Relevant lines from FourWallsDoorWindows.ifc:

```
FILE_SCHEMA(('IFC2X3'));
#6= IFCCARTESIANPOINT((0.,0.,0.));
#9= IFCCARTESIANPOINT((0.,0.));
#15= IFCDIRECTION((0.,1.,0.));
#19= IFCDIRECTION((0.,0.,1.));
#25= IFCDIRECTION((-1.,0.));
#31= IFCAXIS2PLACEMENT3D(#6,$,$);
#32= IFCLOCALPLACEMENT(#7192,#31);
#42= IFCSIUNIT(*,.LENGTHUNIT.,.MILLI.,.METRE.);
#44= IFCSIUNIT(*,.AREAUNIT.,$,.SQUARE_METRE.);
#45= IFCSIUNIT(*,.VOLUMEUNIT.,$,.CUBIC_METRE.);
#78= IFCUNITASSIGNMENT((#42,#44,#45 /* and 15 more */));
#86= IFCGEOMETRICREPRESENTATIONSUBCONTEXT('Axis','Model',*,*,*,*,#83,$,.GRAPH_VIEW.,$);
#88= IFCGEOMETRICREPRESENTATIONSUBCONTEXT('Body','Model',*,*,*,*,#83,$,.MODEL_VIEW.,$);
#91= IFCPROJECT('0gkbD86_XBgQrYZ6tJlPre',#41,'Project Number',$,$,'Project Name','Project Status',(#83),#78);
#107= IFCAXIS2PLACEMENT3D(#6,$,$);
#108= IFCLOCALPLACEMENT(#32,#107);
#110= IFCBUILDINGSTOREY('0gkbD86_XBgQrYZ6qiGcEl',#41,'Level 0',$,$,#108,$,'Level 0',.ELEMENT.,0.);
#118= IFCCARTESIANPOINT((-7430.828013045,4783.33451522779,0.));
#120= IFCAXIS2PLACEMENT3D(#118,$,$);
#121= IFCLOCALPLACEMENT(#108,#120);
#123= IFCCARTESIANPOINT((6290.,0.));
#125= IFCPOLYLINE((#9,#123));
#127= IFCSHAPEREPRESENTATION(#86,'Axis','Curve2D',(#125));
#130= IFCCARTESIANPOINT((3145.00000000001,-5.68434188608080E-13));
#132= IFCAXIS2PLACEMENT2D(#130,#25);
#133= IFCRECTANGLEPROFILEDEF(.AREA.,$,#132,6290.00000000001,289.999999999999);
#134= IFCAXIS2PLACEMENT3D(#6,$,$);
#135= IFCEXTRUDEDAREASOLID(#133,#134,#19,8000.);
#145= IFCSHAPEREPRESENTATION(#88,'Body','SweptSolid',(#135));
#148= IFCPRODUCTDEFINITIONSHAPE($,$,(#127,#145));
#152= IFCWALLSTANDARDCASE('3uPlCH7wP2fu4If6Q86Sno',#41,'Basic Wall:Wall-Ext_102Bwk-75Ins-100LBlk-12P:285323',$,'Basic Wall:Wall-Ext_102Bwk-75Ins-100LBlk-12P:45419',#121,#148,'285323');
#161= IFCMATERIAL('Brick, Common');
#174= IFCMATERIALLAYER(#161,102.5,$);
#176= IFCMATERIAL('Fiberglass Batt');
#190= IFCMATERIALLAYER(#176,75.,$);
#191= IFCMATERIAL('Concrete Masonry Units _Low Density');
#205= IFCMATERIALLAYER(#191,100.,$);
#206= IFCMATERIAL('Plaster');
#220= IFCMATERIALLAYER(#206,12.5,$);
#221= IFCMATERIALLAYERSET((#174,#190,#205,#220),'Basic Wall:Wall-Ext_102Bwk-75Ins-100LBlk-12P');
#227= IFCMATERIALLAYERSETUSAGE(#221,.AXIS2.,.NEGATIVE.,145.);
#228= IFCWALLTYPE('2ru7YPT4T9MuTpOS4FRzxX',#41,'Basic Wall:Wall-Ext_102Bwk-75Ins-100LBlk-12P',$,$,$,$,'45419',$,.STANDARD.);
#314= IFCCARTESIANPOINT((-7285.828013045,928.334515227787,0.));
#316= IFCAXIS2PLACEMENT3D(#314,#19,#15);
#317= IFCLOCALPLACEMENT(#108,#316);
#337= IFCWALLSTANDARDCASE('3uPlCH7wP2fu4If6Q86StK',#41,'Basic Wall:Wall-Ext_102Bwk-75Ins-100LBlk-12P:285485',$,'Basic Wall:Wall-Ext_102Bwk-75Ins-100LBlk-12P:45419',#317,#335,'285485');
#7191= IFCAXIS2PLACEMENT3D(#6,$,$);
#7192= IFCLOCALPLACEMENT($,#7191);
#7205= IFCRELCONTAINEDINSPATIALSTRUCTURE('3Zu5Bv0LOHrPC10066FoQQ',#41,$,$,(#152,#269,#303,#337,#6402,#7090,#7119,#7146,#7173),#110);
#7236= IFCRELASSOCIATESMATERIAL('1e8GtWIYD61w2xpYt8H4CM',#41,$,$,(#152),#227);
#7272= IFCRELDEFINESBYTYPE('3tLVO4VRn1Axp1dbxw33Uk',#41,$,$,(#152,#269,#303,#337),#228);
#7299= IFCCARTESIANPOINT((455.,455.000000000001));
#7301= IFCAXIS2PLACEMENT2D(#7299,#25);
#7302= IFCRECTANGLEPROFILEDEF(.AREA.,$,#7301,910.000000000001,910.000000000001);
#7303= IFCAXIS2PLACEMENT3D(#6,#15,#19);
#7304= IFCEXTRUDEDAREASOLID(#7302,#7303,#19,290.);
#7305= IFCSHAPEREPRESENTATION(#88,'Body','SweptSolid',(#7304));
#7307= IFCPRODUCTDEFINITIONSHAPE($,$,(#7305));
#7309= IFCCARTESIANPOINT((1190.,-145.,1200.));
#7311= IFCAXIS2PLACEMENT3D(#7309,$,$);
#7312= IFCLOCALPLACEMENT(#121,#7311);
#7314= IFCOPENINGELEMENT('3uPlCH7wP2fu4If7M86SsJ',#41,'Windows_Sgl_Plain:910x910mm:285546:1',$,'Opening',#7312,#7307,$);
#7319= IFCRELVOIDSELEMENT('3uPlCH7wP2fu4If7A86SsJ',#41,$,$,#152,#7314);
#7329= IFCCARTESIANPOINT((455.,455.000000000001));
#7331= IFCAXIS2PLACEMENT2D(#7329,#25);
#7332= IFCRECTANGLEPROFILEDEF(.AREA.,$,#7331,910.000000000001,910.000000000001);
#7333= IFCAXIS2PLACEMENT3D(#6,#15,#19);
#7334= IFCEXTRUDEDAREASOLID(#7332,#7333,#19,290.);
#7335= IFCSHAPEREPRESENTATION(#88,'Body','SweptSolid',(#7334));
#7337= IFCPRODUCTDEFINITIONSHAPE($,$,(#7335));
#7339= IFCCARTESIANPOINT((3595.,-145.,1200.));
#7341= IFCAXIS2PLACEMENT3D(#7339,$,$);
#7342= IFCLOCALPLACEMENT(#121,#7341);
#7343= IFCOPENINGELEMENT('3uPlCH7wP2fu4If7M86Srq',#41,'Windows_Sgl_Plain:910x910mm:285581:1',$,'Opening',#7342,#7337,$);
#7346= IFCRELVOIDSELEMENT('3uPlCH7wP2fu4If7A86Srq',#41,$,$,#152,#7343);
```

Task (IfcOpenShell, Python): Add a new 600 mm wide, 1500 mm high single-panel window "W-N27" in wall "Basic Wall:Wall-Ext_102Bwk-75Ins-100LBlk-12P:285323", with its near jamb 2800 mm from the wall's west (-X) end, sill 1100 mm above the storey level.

```python
import numpy as np
import ifcopenshell
import ifcopenshell.api.feature
import ifcopenshell.api.geometry
import ifcopenshell.api.root
import ifcopenshell.api.spatial
import ifcopenshell.api.type
import ifcopenshell.geom
import ifcopenshell.util.element
import ifcopenshell.util.placement
import ifcopenshell.util.representation
import ifcopenshell.util.shape
import ifcopenshell.util.unit

model = ifcopenshell.open("FourWallsDoorWindows.ifc")
unit_scale = ifcopenshell.util.unit.calculate_unit_scale(model)
settings = ifcopenshell.geom.settings()


def volume(element):
    """Net volume in cubic metres, openings subtracted."""
    shape = ifcopenshell.geom.create_shape(settings, element)
    return ifcopenshell.util.shape.get_volume(shape.geometry)


wall = model.by_guid("3uPlCH7wP2fu4If6Q86Sno")
storey = ifcopenshell.util.element.get_container(wall, ifc_class="IfcBuildingStorey")
context = ifcopenshell.util.representation.get_context(model, "Model", "Body", "MODEL_VIEW")
before = volume(wall)

width, height, from_end, sill = 0.6, 1.5, 2.8, 1.1  # metres

# The wall runs along its own X axis, and the end named is its -X end.
wall_shape = ifcopenshell.geom.create_shape(settings, wall)
x, y, z = ifcopenshell.util.shape.get_vertices(wall_shape.geometry).T
start = x.min() + from_end
face, thickness = float(y.min()), float(y.max() - y.min())
wall_matrix = ifcopenshell.util.placement.get_local_placement(wall.ObjectPlacement)
level = ifcopenshell.util.placement.get_local_placement(storey.ObjectPlacement)[2, 3]


def in_wall(x, y):
    """Placement at x, y metres in the wall's axes, at sill height."""
    matrix = wall_matrix.copy()
    matrix[:, 3] = wall_matrix @ np.array([x / unit_scale, y / unit_scale, 0.0, 1.0])
    matrix[2, 3] = level + sill / unit_scale
    return matrix


# Opening: a box that overshoots both wall faces by 50 mm.
opening = ifcopenshell.api.root.create_entity(model, ifc_class="IfcOpeningElement")
box = ifcopenshell.api.geometry.add_wall_representation(
    model, context=context, length=width, height=height, thickness=thickness + 0.1
)
ifcopenshell.api.geometry.assign_representation(model, product=opening, representation=box)
ifcopenshell.api.geometry.edit_object_placement(model, product=opening, matrix=in_wall(start, face - 0.05), is_si=False)
ifcopenshell.api.feature.add_feature(model, feature=opening, element=wall)

window = ifcopenshell.api.root.create_entity(model, ifc_class="IfcWindow", name="W-N27")
window.OverallWidth, window.OverallHeight = width / unit_scale, height / unit_scale
body = ifcopenshell.api.geometry.add_window_representation(
    model,
    context=context,
    overall_width=window.OverallWidth,
    overall_height=window.OverallHeight,
    partition_type="SINGLE_PANEL",
)
ifcopenshell.api.geometry.assign_representation(model, product=window, representation=body)
ifcopenshell.api.spatial.assign_container(model, products=[window], relating_structure=storey)
fills = ifcopenshell.api.feature.add_filling(model, opening=opening, element=window)
fills.OwnerHistory = window.OwnerHistory  # required in IFC2X3

# IFC2X3 keeps the operation on the window style.
style = ifcopenshell.api.root.create_entity(model, ifc_class="IfcWindowStyle", name="W-N27")
style.OperationType, style.ConstructionType = "SINGLE_PANEL", "NOTDEFINED"
style.ParameterTakesPrecedence = style.Sizeable = False
ifcopenshell.api.type.assign_type(model, related_objects=[window], relating_type=style)

# Centre the window in the wall's thickness.
ifcopenshell.api.geometry.edit_object_placement(model, product=window, matrix=in_wall(start, face), is_si=False)
window_shape = ifcopenshell.geom.create_shape(settings, window)
depth = ifcopenshell.util.shape.get_vertices(window_shape.geometry)[:, 1]
offset = face + thickness / 2 - (depth.min() + depth.max()) / 2
ifcopenshell.api.geometry.edit_object_placement(model, product=window, matrix=in_wall(start, offset), is_si=False)

after = volume(wall)

print(f"wall volume {before:.3f} -> {after:.3f} m3")

model.write("FourWallsDoorWindows-out.ifc")
```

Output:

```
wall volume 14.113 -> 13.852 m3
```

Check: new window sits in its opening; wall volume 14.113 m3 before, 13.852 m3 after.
